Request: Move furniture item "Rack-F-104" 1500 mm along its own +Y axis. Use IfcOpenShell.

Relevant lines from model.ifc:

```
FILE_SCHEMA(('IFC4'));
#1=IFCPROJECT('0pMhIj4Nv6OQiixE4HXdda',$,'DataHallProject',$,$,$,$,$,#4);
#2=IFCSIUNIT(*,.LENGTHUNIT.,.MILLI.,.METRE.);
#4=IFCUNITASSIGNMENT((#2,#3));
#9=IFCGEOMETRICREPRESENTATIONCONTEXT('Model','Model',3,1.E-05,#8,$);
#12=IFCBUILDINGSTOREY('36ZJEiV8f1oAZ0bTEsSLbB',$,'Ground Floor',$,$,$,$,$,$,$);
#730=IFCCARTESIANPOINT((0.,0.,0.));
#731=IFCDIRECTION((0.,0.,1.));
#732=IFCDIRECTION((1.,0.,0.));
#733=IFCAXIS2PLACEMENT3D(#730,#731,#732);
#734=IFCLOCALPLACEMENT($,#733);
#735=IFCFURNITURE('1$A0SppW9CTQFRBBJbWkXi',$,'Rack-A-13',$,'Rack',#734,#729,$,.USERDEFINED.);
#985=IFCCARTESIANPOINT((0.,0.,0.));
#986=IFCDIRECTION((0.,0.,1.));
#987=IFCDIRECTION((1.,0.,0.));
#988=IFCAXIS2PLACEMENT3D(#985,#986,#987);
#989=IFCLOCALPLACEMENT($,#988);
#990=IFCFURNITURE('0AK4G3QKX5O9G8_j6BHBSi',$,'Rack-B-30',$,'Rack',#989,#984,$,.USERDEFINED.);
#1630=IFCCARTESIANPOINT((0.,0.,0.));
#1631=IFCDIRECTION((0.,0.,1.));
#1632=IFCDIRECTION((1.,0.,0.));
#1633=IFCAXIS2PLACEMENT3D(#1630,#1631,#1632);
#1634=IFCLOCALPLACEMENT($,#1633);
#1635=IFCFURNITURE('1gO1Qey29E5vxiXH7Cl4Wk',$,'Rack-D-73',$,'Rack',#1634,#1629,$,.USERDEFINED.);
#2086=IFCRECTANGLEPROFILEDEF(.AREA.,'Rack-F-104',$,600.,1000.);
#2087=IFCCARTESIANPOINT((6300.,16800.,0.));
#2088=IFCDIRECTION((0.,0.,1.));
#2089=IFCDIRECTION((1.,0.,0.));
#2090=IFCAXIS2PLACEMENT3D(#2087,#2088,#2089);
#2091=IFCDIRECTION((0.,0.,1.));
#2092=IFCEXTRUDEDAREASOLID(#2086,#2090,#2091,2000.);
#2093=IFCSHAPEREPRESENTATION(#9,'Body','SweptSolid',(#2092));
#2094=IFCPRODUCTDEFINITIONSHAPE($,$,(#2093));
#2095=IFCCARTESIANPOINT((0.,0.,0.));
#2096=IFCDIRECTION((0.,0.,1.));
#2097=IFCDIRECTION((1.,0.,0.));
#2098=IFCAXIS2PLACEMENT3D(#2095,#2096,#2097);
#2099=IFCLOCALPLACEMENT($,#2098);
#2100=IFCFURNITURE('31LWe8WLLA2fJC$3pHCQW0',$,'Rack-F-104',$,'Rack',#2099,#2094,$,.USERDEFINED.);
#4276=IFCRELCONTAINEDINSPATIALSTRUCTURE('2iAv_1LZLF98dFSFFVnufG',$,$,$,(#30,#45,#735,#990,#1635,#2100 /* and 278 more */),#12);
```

```python
import ifcopenshell
import ifcopenshell.api.geometry
import ifcopenshell.util.placement

model = ifcopenshell.open("model.ifc")

item = model.by_guid("31LWe8WLLA2fJC$3pHCQW0")
matrix = ifcopenshell.util.placement.get_local_placement(item.ObjectPlacement)
matrix[:3, 3] += matrix[:3, 1] * 1500.0
ifcopenshell.api.geometry.edit_object_placement(model, product=item, matrix=matrix, is_si=False)

print(ifcopenshell.util.placement.get_local_placement(item.ObjectPlacement).round(3) + 0.0)

model.write("model_v2.ifc")
```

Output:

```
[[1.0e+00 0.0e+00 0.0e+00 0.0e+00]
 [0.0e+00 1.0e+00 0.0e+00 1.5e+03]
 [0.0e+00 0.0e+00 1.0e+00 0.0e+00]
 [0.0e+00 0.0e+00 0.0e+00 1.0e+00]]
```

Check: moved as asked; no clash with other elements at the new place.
